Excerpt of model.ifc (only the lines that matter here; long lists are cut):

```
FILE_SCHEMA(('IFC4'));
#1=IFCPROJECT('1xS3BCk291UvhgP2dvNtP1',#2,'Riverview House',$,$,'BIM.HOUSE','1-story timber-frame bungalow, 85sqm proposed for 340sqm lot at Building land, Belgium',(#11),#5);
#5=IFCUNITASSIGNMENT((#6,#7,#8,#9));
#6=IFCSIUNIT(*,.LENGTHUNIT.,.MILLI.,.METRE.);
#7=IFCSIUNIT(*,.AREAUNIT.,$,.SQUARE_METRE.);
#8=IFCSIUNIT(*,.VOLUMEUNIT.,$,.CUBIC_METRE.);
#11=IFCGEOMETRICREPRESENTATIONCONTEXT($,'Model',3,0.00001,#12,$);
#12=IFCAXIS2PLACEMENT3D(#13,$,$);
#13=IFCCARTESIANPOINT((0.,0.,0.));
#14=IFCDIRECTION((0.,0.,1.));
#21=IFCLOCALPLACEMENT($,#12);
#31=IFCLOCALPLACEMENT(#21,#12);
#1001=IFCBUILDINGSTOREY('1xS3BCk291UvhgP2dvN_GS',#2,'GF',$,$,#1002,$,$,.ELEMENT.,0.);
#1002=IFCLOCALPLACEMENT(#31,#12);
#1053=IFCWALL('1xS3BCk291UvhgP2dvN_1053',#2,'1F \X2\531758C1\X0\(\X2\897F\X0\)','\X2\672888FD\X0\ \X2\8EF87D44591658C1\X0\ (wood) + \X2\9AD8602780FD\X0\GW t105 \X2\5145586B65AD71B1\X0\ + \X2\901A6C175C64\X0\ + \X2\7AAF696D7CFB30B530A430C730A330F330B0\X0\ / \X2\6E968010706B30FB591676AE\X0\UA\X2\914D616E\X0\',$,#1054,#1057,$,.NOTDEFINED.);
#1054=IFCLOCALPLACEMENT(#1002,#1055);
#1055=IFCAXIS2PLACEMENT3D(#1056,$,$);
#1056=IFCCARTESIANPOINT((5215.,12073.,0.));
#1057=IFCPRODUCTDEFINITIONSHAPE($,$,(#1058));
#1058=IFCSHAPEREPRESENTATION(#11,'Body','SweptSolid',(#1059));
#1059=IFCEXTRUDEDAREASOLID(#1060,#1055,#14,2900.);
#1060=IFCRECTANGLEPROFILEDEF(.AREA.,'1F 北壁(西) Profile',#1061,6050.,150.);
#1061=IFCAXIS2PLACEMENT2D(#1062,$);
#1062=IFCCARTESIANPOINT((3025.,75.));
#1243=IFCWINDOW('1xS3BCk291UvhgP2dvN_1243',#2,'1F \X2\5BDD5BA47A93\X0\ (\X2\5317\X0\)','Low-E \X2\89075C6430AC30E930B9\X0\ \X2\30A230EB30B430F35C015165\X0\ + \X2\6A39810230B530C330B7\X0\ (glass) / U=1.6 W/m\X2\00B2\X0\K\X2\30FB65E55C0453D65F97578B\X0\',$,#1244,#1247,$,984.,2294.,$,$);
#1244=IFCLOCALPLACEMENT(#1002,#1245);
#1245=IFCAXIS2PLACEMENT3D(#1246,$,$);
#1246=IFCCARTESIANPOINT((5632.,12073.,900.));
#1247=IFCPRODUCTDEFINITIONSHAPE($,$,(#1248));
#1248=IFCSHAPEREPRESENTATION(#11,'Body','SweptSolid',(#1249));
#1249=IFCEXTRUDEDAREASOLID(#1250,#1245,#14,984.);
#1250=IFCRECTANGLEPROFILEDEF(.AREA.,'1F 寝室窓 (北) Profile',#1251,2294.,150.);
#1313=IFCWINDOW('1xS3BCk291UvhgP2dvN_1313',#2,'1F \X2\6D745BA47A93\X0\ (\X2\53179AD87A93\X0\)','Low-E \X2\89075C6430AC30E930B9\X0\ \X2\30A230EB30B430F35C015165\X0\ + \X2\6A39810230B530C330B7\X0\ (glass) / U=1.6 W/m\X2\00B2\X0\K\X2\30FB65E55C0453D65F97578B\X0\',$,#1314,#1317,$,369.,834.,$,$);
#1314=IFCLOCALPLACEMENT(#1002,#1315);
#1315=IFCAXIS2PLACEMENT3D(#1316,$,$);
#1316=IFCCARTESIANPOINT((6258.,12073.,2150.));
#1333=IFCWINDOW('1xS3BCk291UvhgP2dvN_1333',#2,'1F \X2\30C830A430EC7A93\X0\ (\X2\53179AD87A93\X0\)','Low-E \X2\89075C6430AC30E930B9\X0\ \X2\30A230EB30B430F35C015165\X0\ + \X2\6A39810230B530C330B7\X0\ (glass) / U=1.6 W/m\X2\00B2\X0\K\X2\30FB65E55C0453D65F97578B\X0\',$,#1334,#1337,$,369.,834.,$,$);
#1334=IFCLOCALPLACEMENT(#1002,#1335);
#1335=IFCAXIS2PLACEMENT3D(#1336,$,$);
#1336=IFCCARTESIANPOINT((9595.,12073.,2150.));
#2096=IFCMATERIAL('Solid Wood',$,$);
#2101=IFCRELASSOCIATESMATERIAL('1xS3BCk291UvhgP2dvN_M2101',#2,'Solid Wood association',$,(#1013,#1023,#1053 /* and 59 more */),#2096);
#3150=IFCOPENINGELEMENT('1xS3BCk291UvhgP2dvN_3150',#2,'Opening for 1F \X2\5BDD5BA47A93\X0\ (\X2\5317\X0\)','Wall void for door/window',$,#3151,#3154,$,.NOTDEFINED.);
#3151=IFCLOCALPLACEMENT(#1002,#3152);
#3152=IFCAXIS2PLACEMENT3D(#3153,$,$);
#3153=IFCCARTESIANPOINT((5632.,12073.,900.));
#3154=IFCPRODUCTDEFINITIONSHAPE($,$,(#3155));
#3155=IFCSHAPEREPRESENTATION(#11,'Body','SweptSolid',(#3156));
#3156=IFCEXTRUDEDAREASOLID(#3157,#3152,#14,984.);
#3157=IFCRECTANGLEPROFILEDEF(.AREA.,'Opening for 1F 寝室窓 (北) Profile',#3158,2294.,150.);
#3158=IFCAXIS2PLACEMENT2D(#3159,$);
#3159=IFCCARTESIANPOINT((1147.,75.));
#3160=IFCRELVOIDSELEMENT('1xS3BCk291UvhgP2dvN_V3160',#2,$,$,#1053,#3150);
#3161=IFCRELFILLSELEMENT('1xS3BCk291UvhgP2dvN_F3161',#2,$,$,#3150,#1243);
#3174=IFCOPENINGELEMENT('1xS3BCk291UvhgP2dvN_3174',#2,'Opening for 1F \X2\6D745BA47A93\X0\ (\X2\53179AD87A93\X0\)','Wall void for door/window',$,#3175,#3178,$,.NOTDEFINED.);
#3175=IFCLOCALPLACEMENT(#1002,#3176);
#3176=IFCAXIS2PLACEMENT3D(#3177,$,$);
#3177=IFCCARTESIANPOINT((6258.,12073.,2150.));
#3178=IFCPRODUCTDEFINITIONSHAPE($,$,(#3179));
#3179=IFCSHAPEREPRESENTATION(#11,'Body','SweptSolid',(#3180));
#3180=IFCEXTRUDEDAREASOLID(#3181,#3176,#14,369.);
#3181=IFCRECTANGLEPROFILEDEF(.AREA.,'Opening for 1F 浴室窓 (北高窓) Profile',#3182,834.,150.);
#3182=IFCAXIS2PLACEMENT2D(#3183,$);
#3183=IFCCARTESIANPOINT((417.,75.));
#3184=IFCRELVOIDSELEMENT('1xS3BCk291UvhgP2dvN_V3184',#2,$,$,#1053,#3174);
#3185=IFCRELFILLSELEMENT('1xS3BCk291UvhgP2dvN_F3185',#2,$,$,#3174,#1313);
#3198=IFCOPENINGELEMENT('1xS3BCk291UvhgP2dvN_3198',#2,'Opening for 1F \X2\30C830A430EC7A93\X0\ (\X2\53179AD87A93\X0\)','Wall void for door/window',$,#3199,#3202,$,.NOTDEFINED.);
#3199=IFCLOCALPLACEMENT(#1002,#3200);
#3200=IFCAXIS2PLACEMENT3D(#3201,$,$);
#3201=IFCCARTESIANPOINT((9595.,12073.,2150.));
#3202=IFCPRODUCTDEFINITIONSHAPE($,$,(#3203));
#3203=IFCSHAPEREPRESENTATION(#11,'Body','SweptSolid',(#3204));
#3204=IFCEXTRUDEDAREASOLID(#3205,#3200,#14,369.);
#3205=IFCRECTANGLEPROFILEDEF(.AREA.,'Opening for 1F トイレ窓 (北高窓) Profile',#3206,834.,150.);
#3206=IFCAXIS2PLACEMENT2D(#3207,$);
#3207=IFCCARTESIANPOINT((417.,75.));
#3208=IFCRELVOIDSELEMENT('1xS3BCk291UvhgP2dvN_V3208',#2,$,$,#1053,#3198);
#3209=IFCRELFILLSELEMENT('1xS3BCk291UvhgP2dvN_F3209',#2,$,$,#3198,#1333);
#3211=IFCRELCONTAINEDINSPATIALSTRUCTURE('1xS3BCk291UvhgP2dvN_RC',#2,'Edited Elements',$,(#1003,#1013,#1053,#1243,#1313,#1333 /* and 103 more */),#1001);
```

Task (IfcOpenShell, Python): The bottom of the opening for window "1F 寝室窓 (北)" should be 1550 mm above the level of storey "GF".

```python
import numpy as np
import ifcopenshell
import ifcopenshell.api.geometry
import ifcopenshell.geom
import ifcopenshell.util.element
import ifcopenshell.util.placement
import ifcopenshell.util.shape
import ifcopenshell.util.unit

model = ifcopenshell.open("model.ifc")
unit_scale = ifcopenshell.util.unit.calculate_unit_scale(model)

window = model.by_guid("1xS3BCk291UvhgP2dvN_1243")
opening = window.FillsVoids[0].RelatingOpeningElement
storey = ifcopenshell.util.element.get_container(window, ifc_class="IfcBuildingStorey")
level = ifcopenshell.util.placement.get_local_placement(storey.ObjectPlacement)[2, 3]

# The opening's origin need not be at the sill, so measure its lowest point.
shape = ifcopenshell.geom.create_shape(ifcopenshell.geom.settings(), opening)
bottom = ifcopenshell.util.shape.get_shape_bottom_elevation(shape, shape.geometry) / unit_scale
dz = level + 1.55 / unit_scale - bottom

shift = np.array([0.0, 0.0, dz])
# The window is not placed relative to its opening, so move both.
for product in (opening, window):
    matrix = ifcopenshell.util.placement.get_local_placement(product.ObjectPlacement)
    matrix[:3, 3] += shift
    ifcopenshell.api.geometry.edit_object_placement(model, product=product, matrix=matrix, is_si=False)

print(f"moved by {dz * unit_scale:+.3f} m")

model.write("model_updated.ifc")
```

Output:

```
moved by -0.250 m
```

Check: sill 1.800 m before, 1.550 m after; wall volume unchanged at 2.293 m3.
